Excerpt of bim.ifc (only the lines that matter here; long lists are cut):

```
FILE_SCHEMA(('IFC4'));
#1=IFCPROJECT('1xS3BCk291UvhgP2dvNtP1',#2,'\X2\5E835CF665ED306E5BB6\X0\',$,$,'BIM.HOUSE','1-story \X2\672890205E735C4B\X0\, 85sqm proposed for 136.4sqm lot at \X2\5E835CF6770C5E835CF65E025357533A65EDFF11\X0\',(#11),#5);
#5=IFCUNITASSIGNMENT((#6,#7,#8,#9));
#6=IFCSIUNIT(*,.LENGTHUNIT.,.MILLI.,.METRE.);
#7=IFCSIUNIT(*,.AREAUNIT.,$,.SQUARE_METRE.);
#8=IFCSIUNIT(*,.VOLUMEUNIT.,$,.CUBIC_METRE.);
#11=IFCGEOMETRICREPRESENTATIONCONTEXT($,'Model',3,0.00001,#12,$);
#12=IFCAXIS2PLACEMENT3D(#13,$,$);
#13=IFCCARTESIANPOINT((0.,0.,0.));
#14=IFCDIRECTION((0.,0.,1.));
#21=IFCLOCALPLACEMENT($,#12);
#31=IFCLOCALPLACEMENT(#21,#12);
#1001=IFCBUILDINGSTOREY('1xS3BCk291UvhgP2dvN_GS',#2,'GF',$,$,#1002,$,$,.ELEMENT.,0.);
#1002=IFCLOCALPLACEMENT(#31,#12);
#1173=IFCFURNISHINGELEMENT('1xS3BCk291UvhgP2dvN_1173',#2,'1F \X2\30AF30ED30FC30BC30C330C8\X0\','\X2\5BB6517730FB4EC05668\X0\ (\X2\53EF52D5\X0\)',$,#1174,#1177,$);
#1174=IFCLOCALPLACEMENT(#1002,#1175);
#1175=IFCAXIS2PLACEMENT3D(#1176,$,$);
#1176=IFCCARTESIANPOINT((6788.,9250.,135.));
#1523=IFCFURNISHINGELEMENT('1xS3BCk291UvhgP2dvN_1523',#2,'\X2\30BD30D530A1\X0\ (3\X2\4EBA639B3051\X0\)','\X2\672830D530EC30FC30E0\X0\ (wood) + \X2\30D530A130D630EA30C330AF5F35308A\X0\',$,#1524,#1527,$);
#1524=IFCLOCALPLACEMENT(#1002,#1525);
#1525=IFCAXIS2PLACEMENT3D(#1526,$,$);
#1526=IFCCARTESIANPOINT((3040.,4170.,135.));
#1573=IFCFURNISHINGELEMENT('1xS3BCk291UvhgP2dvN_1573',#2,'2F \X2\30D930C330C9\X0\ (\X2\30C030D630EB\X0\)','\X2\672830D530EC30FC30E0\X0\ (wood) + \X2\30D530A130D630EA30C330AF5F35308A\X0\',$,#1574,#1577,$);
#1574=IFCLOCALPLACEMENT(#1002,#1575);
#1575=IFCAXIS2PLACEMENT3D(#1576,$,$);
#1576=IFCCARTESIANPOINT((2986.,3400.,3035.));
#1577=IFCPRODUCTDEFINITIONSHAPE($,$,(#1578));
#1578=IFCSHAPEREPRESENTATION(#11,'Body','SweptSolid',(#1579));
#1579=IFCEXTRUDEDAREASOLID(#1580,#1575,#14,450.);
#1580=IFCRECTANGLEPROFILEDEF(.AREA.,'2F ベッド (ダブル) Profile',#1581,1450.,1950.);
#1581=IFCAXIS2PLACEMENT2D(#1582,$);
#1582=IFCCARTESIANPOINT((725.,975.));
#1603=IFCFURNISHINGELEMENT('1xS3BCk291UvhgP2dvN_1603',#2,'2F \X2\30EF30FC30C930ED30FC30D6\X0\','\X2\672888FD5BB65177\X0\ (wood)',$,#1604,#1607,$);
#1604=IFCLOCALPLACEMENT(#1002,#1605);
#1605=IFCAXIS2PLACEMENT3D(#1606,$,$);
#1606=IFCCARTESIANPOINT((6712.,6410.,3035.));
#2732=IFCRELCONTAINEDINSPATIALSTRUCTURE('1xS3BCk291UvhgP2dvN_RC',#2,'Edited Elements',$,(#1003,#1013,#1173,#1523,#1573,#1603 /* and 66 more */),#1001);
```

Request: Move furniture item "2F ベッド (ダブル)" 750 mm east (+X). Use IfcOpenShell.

```python
import ifcopenshell
import ifcopenshell.api.geometry
import ifcopenshell.util.placement

model = ifcopenshell.open("bim.ifc")

item = model.by_id(1573)
matrix = ifcopenshell.util.placement.get_local_placement(item.ObjectPlacement)
matrix[0, 3] += 750.0
ifcopenshell.api.geometry.edit_object_placement(model, product=item, matrix=matrix, is_si=False)

print(ifcopenshell.util.placement.get_local_placement(item.ObjectPlacement).round(3) + 0.0)

model.write("bim_updated.ifc")
```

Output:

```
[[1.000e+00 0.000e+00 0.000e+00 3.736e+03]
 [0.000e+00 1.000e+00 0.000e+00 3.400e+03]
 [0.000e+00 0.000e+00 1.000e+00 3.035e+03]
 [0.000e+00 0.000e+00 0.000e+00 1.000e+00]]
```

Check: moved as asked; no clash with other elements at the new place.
